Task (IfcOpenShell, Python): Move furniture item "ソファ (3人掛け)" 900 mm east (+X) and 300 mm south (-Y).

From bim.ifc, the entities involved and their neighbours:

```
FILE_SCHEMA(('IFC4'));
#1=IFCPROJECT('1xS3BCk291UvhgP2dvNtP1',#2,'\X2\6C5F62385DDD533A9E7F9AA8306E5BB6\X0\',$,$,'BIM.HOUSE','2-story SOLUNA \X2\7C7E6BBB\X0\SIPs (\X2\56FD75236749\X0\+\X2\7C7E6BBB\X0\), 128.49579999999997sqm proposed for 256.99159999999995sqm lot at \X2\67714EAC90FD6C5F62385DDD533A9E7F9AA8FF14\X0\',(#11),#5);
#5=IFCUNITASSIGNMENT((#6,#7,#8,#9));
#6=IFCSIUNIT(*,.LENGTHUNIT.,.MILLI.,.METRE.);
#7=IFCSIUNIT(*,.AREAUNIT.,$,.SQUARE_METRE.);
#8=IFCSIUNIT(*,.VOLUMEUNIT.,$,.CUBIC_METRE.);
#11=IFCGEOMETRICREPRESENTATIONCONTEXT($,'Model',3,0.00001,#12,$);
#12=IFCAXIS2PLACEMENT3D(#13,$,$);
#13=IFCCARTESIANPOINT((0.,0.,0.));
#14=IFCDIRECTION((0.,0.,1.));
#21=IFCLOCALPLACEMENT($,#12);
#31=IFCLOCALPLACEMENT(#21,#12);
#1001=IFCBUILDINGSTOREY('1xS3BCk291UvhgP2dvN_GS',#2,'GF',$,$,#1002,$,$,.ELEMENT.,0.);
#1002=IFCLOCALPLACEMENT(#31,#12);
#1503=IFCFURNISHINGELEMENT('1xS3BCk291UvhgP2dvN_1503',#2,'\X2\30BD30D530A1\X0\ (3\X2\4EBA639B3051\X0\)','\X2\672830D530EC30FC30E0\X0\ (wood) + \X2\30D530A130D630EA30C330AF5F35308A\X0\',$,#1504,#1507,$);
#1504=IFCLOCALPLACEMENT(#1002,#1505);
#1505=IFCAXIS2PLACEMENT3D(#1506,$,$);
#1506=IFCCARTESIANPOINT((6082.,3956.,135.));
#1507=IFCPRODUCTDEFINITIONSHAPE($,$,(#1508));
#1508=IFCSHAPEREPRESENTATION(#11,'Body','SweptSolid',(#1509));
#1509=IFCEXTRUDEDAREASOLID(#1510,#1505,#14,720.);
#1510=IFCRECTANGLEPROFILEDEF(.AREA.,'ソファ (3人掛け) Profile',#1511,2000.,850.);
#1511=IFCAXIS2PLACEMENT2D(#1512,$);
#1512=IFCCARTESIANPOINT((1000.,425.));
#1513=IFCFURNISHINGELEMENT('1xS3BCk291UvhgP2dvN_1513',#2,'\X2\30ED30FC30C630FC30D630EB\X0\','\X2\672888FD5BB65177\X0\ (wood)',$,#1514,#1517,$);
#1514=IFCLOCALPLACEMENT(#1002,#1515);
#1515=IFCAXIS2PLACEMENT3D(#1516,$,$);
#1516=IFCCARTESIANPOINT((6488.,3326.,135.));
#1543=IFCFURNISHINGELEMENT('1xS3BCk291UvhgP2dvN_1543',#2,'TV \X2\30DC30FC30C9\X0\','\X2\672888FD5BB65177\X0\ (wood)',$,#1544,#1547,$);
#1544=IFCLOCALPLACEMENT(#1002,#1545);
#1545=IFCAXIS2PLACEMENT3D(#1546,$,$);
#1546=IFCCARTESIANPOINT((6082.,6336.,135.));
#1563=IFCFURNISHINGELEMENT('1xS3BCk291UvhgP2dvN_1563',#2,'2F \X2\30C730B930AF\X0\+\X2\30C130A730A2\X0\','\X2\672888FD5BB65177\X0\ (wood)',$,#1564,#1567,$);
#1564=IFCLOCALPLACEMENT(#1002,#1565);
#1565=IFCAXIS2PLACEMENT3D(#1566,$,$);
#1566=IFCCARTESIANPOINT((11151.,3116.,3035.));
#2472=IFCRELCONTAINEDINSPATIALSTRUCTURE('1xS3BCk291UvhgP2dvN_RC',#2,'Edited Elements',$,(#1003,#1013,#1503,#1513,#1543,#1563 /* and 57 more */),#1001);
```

```python
import ifcopenshell
import ifcopenshell.api.geometry
import ifcopenshell.util.placement
import ifcopenshell.util.unit

model = ifcopenshell.open("bim.ifc")
unit_scale = ifcopenshell.util.unit.calculate_unit_scale(model)

item = model.by_guid("1xS3BCk291UvhgP2dvN_1503")
matrix = ifcopenshell.util.placement.get_local_placement(item.ObjectPlacement)
matrix[0, 3] += 0.9 / unit_scale
matrix[1, 3] -= 0.3 / unit_scale
ifcopenshell.api.geometry.edit_object_placement(model, product=item, matrix=matrix, is_si=False)

print(ifcopenshell.util.placement.get_local_placement(item.ObjectPlacement).round(3) + 0.0)

model.write("bim_v2.ifc")
```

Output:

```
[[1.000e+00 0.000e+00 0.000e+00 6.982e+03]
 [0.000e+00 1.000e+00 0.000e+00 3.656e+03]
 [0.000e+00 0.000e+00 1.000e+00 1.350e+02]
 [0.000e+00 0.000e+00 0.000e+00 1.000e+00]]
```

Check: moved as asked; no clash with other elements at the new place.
